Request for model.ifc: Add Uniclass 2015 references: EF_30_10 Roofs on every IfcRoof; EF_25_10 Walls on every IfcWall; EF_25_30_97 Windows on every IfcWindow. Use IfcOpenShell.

First a look at what the model holds.

```python
import ifcopenshell

model = ifcopenshell.open("model.ifc")
print(model.schema)
print("classifications:", [c.Name for c in model.by_type("IfcClassification")])
for ifc_class in ("IfcDoor", "IfcRoof", "IfcStair", "IfcWall", "IfcWindow"):
    print(ifc_class, len(model.by_type(ifc_class)))
```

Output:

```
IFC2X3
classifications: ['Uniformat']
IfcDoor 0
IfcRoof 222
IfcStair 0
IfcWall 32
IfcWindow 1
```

```python
import ifcopenshell
import ifcopenshell.api.classification

model = ifcopenshell.open("model.ifc")

# IFC2X3 requires Source and Edition and has no link from the project to the system.
system = model.create_entity("IfcClassification", Source="NBS", Edition="2015", Name="Uniclass 2015")

codes = {
    "IfcRoof": ("EF_30_10", "Roofs"),
    "IfcWall": ("EF_25_10", "Walls"),
    "IfcWindow": ("EF_25_30_97", "Windows"),
}
for ifc_class, (code, name) in codes.items():
    products = model.by_type(ifc_class)
    ifcopenshell.api.classification.add_reference(
        model, products=products, classification=system, identification=code, name=name
    )
    print(code, len(products))

model.write("model_v2.ifc")
```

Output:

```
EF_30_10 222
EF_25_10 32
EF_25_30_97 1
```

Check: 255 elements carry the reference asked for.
